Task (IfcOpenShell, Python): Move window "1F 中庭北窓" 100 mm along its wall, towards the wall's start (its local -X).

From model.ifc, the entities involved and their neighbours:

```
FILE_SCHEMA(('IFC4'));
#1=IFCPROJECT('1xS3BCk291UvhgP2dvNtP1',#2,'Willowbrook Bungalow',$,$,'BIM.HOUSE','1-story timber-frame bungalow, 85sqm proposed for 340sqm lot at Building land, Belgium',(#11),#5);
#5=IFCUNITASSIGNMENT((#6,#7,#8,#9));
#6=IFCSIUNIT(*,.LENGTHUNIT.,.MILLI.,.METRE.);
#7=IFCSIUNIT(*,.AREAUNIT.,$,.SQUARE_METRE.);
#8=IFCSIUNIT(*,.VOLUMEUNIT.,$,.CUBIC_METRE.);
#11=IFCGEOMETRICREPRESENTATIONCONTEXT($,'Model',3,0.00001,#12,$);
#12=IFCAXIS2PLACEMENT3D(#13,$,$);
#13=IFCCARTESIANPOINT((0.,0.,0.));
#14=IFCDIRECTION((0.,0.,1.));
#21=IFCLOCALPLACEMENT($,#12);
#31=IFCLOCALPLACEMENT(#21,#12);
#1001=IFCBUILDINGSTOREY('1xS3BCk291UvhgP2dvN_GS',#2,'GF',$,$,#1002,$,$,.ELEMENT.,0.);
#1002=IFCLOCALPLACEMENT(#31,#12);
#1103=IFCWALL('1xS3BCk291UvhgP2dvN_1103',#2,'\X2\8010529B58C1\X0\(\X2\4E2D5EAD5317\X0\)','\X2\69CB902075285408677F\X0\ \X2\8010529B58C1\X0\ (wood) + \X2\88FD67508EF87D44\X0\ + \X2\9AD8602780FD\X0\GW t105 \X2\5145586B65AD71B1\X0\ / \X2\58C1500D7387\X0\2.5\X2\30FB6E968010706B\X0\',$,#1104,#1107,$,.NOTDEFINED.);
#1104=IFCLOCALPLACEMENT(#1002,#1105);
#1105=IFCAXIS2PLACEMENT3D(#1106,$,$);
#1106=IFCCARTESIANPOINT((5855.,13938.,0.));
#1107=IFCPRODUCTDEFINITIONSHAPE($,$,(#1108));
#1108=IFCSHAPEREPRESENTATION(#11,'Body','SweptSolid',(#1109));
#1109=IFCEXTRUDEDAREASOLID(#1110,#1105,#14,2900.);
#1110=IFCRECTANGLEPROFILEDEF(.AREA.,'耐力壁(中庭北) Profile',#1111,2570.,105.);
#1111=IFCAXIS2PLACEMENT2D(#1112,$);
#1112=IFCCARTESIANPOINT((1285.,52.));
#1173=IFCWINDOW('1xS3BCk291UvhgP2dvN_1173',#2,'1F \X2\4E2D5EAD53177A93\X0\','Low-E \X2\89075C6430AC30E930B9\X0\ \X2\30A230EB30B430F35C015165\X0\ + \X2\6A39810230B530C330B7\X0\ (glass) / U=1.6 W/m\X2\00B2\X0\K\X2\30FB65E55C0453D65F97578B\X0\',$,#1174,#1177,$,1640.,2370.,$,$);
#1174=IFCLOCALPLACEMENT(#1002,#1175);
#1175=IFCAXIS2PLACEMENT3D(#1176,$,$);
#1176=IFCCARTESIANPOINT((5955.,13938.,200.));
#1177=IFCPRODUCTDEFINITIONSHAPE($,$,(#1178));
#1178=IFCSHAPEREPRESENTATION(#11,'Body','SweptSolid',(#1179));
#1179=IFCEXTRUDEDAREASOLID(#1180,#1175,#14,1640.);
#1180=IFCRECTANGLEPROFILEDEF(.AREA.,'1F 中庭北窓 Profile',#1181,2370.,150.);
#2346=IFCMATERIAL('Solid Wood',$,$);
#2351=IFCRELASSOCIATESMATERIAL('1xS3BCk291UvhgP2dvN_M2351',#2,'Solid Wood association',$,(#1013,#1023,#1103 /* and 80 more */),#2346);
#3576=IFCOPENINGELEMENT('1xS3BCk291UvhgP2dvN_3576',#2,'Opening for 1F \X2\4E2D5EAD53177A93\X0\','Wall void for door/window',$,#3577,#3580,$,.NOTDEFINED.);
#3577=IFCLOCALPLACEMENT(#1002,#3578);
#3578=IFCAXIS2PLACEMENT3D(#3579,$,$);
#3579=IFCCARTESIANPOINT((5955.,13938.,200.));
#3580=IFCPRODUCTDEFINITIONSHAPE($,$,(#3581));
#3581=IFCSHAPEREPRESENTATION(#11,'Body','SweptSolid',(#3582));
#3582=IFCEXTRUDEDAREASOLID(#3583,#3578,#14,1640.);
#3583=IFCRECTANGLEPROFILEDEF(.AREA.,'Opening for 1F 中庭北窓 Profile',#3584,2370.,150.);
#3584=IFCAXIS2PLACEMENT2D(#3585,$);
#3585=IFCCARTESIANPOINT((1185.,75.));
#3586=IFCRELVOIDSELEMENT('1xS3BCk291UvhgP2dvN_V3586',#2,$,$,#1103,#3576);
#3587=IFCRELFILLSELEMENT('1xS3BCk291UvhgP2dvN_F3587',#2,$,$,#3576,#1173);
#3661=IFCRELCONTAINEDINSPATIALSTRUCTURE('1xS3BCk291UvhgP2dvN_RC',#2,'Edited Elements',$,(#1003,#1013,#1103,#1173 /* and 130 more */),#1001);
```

```python
import ifcopenshell
import ifcopenshell.api.geometry
import ifcopenshell.util.placement
import ifcopenshell.util.unit

model = ifcopenshell.open("model.ifc")
unit_scale = ifcopenshell.util.unit.calculate_unit_scale(model)

window = model.by_guid("1xS3BCk291UvhgP2dvN_1173")
opening = window.FillsVoids[0].RelatingOpeningElement
wall = opening.VoidsElements[0].RelatingBuildingElement

wall_matrix = ifcopenshell.util.placement.get_local_placement(wall.ObjectPlacement)
shift = wall_matrix[:3, 0] * -0.1 / unit_scale
before = ifcopenshell.util.placement.get_local_placement(window.ObjectPlacement)[:3, 3].copy()

# The window is not placed relative to its opening, so move both.
for product in (opening, window):
    matrix = ifcopenshell.util.placement.get_local_placement(product.ObjectPlacement)
    matrix[:3, 3] += shift
    ifcopenshell.api.geometry.edit_object_placement(model, product=product, matrix=matrix, is_si=False)

after = ifcopenshell.util.placement.get_local_placement(window.ObjectPlacement)[:3, 3]
print("window moved by", (after - before).round(3) + 0.0)

model.write("model_rev.ifc")
```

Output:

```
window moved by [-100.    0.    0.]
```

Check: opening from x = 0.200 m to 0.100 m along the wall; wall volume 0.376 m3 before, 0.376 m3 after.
